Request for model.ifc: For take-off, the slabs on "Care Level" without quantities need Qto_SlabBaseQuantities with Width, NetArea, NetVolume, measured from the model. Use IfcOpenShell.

First a look at what the model holds.

```python
import ifcopenshell
import ifcopenshell.util.element
import ifcopenshell.util.unit

model = ifcopenshell.open("model.ifc")
print(model.schema)
for unit_type in ("LENGTHUNIT", "AREAUNIT", "VOLUMEUNIT"):
    print(unit_type, ifcopenshell.util.unit.calculate_unit_scale(model, unit_type))
storey = next(s for s in model.by_type("IfcBuildingStorey") if s.Name == "Care Level")
slabs = [e for e in ifcopenshell.util.element.get_decomposition(storey) if e.is_a("IfcSlab")]
for e in sorted(slabs, key=lambda e: e.id()):
    print(e.id(), e.is_a(), e.Name, list(ifcopenshell.util.element.get_psets(e, qtos_only=True)), sep=" | ")
```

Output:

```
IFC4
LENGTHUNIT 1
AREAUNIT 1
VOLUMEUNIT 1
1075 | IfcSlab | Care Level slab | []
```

```python
import ifcopenshell
import ifcopenshell.api.pset
import ifcopenshell.geom
import ifcopenshell.util.element
import ifcopenshell.util.shape
import ifcopenshell.util.unit

model = ifcopenshell.open("model.ifc")
unit_scale = ifcopenshell.util.unit.calculate_unit_scale(model)
area_scale = ifcopenshell.util.unit.calculate_unit_scale(model, "AREAUNIT")
volume_scale = ifcopenshell.util.unit.calculate_unit_scale(model, "VOLUMEUNIT")
settings = ifcopenshell.geom.settings()

storey = next(s for s in model.by_type("IfcBuildingStorey") if s.Name == "Care Level")
slabs = [e for e in ifcopenshell.util.element.get_decomposition(storey) if e.is_a("IfcSlab")]

for e in sorted(slabs, key=lambda e: e.id()):
    if ifcopenshell.util.element.get_psets(e, qtos_only=True, should_inherit=False):
        continue
    # Geometry comes back in metres, in the element's own axes.
    shape = ifcopenshell.geom.create_shape(settings, e)
    values = {
        "Width": ifcopenshell.util.shape.get_z(shape.geometry) / unit_scale,
        "NetArea": ifcopenshell.util.shape.get_footprint_area(shape.geometry) / area_scale,
        "NetVolume": ifcopenshell.util.shape.get_volume(shape.geometry) / volume_scale,
    }
    qto = ifcopenshell.api.pset.add_qto(model, product=e, name="Qto_SlabBaseQuantities")
    ifcopenshell.api.pset.edit_qto(model, qto=qto, properties=values)
    print(e.id(), {k: round(v, 3) for k, v in values.items()})

model.write("model_edited.ifc")
```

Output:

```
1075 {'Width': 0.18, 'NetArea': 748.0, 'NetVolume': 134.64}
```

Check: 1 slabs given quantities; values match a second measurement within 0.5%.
